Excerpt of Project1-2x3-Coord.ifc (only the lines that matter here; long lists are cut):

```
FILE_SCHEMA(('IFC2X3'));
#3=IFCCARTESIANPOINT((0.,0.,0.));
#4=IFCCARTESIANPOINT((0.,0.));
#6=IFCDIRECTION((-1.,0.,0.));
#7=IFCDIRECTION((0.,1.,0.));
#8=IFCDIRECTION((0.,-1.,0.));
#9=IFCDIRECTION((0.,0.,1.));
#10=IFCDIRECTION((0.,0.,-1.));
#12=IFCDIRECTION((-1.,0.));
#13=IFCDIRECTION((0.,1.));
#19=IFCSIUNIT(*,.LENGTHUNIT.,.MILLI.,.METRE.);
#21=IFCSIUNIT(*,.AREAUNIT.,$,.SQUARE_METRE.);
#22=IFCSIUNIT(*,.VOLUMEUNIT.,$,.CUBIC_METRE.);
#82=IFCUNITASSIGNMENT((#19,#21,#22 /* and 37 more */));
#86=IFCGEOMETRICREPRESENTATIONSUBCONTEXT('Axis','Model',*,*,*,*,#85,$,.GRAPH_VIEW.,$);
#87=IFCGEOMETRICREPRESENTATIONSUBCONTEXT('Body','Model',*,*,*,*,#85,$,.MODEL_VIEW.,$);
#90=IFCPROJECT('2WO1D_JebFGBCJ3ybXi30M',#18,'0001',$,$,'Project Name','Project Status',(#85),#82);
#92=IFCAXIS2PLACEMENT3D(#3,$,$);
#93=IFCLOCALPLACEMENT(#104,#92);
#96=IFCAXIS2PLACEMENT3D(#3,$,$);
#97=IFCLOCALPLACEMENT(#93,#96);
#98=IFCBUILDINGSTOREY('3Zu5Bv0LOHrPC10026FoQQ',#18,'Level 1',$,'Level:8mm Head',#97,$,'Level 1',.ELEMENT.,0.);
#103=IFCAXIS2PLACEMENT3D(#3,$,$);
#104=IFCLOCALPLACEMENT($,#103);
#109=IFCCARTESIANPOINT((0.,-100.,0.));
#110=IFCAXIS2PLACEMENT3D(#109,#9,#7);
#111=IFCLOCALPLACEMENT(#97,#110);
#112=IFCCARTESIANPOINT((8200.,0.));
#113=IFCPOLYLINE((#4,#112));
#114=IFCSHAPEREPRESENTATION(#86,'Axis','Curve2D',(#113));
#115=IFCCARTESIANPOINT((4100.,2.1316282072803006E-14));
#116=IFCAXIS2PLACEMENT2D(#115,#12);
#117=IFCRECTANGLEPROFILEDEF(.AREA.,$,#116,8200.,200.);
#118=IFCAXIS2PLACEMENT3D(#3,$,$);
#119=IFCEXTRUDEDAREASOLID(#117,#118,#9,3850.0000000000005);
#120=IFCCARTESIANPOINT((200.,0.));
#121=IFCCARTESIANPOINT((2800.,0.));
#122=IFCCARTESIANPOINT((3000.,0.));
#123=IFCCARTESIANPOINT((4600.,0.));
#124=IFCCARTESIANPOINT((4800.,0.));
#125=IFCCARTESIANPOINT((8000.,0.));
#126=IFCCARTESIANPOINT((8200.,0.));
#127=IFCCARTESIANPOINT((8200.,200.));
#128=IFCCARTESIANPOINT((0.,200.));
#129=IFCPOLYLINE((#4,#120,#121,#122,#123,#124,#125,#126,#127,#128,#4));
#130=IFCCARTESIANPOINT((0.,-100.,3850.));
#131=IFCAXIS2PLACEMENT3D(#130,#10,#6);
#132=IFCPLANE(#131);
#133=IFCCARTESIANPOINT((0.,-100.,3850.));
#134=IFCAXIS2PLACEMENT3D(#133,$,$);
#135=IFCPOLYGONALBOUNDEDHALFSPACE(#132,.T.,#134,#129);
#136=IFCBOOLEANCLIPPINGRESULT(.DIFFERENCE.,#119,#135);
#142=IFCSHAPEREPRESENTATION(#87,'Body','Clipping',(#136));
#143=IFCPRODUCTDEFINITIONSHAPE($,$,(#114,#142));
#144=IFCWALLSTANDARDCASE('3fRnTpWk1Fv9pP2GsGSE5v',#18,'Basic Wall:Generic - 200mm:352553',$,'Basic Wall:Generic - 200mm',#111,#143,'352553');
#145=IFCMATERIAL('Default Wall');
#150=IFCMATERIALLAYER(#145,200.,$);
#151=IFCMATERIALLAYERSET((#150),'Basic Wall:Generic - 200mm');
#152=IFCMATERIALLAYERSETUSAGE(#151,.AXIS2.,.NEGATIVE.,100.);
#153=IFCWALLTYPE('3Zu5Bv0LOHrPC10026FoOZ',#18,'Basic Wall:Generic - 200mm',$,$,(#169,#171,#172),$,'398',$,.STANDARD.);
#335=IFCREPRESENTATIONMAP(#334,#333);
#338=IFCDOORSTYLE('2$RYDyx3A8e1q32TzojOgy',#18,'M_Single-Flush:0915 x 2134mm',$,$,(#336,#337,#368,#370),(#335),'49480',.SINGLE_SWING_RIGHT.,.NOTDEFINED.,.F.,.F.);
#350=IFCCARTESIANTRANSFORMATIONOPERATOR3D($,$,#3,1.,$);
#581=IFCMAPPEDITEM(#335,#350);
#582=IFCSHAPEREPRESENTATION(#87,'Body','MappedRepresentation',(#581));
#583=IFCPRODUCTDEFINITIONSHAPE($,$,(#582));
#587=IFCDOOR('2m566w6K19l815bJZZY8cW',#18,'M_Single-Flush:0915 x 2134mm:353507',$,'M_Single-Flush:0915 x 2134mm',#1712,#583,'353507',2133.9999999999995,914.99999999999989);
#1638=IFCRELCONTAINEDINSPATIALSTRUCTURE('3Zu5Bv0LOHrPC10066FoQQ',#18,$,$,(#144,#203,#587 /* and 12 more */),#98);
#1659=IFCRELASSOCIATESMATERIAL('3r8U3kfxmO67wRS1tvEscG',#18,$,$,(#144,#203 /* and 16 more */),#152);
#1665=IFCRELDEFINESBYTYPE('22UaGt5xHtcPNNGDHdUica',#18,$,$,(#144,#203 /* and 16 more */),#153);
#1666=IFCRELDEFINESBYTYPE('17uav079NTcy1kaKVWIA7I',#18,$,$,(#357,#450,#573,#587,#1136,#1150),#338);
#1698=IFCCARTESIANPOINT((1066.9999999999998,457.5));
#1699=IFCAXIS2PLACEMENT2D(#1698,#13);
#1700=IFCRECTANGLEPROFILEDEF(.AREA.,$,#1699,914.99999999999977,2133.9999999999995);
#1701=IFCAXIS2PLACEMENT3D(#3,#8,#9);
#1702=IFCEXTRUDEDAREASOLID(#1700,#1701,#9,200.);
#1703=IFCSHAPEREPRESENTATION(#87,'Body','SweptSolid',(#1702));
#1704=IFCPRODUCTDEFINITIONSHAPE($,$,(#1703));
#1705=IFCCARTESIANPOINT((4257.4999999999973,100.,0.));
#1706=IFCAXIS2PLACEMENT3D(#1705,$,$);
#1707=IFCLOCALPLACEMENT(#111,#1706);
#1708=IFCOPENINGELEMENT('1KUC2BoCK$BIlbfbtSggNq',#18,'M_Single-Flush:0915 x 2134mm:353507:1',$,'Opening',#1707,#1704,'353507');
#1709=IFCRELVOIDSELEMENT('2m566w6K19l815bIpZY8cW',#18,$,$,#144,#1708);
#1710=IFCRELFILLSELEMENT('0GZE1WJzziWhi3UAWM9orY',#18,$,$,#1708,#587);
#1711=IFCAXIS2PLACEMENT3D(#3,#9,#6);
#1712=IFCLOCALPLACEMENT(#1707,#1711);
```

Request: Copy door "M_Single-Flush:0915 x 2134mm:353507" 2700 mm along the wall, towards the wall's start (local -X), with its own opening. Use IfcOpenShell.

```python
import ifcopenshell
import ifcopenshell.api.feature
import ifcopenshell.api.geometry
import ifcopenshell.api.root
import ifcopenshell.geom
import ifcopenshell.util.element
import ifcopenshell.util.placement
import ifcopenshell.util.shape
import ifcopenshell.util.unit

model = ifcopenshell.open("Project1-2x3-Coord.ifc")
unit_scale = ifcopenshell.util.unit.calculate_unit_scale(model)
settings = ifcopenshell.geom.settings()


def volume(element):
    """Net volume in cubic metres, openings subtracted."""
    shape = ifcopenshell.geom.create_shape(settings, element)
    return ifcopenshell.util.shape.get_volume(shape.geometry)


def reuse_history(source, copy):
    """copy_class also copies each property set's owner history, people and application; keep the originals."""
    for rel in copy.IsDefinedBy:
        if rel.is_a("IfcRelDefinesByProperties") and (history := rel.RelatingPropertyDefinition.OwnerHistory):
            rel.RelatingPropertyDefinition.OwnerHistory = source.OwnerHistory
            ifcopenshell.util.element.remove_deep2(model, history)


door = model.by_guid("2m566w6K19l815bJZZY8cW")
opening = door.FillsVoids[0].RelatingOpeningElement
wall = opening.VoidsElements[0].RelatingBuildingElement
before = volume(wall)
shift = ifcopenshell.util.placement.get_local_placement(wall.ObjectPlacement)[:3, 0] * -2.7 / unit_scale

# copy_class copies the void relationship, type, container and properties, but no geometry.
new_opening = ifcopenshell.api.root.copy_class(model, product=opening)
new_opening.Representation = ifcopenshell.util.element.copy_deep(
    model, opening.Representation, exclude=["IfcGeometricRepresentationContext", "IfcRepresentationMap"]
)
new_opening.Name = "M_Single-Flush:0915 x 2134mm"
new_opening.Tag = None
new_door = ifcopenshell.api.root.copy_class(model, product=door)
new_door.Representation = ifcopenshell.util.element.copy_deep(
    model, door.Representation, exclude=["IfcGeometricRepresentationContext", "IfcRepresentationMap"]
)
new_door.Name = "M_Single-Flush:0915 x 2134mm"
new_door.Tag = None
reuse_history(door, new_door)
fills = ifcopenshell.api.feature.add_filling(model, opening=new_opening, element=new_door)
fills.OwnerHistory = new_door.OwnerHistory  # required in IFC2X3

for old, new in ((opening, new_opening), (door, new_door)):
    matrix = ifcopenshell.util.placement.get_local_placement(old.ObjectPlacement)
    matrix[:3, 3] += shift
    ifcopenshell.api.geometry.edit_object_placement(model, product=new, matrix=matrix, is_si=False)

after = volume(wall)

print(f"wall volume {before:.3f} -> {after:.3f} m3")

model.write("Project1-2x3-Coord_updated.ifc")
```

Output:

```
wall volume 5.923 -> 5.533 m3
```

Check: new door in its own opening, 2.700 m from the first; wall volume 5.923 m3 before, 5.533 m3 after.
